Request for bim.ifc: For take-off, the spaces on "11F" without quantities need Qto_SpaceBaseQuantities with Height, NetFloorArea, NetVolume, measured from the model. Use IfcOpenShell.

First a look at what the model holds.

```python
import ifcopenshell
import ifcopenshell.util.element
import ifcopenshell.util.unit

model = ifcopenshell.open("bim.ifc")
print(model.schema)
for unit_type in ("LENGTHUNIT", "AREAUNIT", "VOLUMEUNIT"):
    print(unit_type, ifcopenshell.util.unit.calculate_unit_scale(model, unit_type))
storey = next(s for s in model.by_type("IfcBuildingStorey") if s.Name == "11F")
spaces = [e for e in ifcopenshell.util.element.get_decomposition(storey) if e.is_a("IfcSpace")]
for e in sorted(spaces, key=lambda e: e.id()):
    print(e.id(), e.is_a(), e.Name, list(ifcopenshell.util.element.get_psets(e, qtos_only=True)), sep=" | ")
```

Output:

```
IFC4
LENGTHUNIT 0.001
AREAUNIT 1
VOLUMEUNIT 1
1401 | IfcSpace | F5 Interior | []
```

```python
import ifcopenshell
import ifcopenshell.api.pset
import ifcopenshell.geom
import ifcopenshell.util.element
import ifcopenshell.util.shape
import ifcopenshell.util.unit

model = ifcopenshell.open("bim.ifc")
unit_scale = ifcopenshell.util.unit.calculate_unit_scale(model)
area_scale = ifcopenshell.util.unit.calculate_unit_scale(model, "AREAUNIT")
volume_scale = ifcopenshell.util.unit.calculate_unit_scale(model, "VOLUMEUNIT")
settings = ifcopenshell.geom.settings()

storey = next(s for s in model.by_type("IfcBuildingStorey") if s.Name == "11F")
spaces = [e for e in ifcopenshell.util.element.get_decomposition(storey) if e.is_a("IfcSpace")]

for e in sorted(spaces, key=lambda e: e.id()):
    if ifcopenshell.util.element.get_psets(e, qtos_only=True, should_inherit=False):
        continue
    # Geometry comes back in metres, in the element's own axes.
    shape = ifcopenshell.geom.create_shape(settings, e)
    values = {
        "Height": ifcopenshell.util.shape.get_z(shape.geometry) / unit_scale,
        "NetFloorArea": ifcopenshell.util.shape.get_footprint_area(shape.geometry) / area_scale,
        "NetVolume": ifcopenshell.util.shape.get_volume(shape.geometry) / volume_scale,
    }
    qto = ifcopenshell.api.pset.add_qto(model, product=e, name="Qto_SpaceBaseQuantities")
    ifcopenshell.api.pset.edit_qto(model, qto=qto, properties=values)
    print(e.id(), {k: round(v, 3) for k, v in values.items()})

model.write("bim_rev.ifc")
```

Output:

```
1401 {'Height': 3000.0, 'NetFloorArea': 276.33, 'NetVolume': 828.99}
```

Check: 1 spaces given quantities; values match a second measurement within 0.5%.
